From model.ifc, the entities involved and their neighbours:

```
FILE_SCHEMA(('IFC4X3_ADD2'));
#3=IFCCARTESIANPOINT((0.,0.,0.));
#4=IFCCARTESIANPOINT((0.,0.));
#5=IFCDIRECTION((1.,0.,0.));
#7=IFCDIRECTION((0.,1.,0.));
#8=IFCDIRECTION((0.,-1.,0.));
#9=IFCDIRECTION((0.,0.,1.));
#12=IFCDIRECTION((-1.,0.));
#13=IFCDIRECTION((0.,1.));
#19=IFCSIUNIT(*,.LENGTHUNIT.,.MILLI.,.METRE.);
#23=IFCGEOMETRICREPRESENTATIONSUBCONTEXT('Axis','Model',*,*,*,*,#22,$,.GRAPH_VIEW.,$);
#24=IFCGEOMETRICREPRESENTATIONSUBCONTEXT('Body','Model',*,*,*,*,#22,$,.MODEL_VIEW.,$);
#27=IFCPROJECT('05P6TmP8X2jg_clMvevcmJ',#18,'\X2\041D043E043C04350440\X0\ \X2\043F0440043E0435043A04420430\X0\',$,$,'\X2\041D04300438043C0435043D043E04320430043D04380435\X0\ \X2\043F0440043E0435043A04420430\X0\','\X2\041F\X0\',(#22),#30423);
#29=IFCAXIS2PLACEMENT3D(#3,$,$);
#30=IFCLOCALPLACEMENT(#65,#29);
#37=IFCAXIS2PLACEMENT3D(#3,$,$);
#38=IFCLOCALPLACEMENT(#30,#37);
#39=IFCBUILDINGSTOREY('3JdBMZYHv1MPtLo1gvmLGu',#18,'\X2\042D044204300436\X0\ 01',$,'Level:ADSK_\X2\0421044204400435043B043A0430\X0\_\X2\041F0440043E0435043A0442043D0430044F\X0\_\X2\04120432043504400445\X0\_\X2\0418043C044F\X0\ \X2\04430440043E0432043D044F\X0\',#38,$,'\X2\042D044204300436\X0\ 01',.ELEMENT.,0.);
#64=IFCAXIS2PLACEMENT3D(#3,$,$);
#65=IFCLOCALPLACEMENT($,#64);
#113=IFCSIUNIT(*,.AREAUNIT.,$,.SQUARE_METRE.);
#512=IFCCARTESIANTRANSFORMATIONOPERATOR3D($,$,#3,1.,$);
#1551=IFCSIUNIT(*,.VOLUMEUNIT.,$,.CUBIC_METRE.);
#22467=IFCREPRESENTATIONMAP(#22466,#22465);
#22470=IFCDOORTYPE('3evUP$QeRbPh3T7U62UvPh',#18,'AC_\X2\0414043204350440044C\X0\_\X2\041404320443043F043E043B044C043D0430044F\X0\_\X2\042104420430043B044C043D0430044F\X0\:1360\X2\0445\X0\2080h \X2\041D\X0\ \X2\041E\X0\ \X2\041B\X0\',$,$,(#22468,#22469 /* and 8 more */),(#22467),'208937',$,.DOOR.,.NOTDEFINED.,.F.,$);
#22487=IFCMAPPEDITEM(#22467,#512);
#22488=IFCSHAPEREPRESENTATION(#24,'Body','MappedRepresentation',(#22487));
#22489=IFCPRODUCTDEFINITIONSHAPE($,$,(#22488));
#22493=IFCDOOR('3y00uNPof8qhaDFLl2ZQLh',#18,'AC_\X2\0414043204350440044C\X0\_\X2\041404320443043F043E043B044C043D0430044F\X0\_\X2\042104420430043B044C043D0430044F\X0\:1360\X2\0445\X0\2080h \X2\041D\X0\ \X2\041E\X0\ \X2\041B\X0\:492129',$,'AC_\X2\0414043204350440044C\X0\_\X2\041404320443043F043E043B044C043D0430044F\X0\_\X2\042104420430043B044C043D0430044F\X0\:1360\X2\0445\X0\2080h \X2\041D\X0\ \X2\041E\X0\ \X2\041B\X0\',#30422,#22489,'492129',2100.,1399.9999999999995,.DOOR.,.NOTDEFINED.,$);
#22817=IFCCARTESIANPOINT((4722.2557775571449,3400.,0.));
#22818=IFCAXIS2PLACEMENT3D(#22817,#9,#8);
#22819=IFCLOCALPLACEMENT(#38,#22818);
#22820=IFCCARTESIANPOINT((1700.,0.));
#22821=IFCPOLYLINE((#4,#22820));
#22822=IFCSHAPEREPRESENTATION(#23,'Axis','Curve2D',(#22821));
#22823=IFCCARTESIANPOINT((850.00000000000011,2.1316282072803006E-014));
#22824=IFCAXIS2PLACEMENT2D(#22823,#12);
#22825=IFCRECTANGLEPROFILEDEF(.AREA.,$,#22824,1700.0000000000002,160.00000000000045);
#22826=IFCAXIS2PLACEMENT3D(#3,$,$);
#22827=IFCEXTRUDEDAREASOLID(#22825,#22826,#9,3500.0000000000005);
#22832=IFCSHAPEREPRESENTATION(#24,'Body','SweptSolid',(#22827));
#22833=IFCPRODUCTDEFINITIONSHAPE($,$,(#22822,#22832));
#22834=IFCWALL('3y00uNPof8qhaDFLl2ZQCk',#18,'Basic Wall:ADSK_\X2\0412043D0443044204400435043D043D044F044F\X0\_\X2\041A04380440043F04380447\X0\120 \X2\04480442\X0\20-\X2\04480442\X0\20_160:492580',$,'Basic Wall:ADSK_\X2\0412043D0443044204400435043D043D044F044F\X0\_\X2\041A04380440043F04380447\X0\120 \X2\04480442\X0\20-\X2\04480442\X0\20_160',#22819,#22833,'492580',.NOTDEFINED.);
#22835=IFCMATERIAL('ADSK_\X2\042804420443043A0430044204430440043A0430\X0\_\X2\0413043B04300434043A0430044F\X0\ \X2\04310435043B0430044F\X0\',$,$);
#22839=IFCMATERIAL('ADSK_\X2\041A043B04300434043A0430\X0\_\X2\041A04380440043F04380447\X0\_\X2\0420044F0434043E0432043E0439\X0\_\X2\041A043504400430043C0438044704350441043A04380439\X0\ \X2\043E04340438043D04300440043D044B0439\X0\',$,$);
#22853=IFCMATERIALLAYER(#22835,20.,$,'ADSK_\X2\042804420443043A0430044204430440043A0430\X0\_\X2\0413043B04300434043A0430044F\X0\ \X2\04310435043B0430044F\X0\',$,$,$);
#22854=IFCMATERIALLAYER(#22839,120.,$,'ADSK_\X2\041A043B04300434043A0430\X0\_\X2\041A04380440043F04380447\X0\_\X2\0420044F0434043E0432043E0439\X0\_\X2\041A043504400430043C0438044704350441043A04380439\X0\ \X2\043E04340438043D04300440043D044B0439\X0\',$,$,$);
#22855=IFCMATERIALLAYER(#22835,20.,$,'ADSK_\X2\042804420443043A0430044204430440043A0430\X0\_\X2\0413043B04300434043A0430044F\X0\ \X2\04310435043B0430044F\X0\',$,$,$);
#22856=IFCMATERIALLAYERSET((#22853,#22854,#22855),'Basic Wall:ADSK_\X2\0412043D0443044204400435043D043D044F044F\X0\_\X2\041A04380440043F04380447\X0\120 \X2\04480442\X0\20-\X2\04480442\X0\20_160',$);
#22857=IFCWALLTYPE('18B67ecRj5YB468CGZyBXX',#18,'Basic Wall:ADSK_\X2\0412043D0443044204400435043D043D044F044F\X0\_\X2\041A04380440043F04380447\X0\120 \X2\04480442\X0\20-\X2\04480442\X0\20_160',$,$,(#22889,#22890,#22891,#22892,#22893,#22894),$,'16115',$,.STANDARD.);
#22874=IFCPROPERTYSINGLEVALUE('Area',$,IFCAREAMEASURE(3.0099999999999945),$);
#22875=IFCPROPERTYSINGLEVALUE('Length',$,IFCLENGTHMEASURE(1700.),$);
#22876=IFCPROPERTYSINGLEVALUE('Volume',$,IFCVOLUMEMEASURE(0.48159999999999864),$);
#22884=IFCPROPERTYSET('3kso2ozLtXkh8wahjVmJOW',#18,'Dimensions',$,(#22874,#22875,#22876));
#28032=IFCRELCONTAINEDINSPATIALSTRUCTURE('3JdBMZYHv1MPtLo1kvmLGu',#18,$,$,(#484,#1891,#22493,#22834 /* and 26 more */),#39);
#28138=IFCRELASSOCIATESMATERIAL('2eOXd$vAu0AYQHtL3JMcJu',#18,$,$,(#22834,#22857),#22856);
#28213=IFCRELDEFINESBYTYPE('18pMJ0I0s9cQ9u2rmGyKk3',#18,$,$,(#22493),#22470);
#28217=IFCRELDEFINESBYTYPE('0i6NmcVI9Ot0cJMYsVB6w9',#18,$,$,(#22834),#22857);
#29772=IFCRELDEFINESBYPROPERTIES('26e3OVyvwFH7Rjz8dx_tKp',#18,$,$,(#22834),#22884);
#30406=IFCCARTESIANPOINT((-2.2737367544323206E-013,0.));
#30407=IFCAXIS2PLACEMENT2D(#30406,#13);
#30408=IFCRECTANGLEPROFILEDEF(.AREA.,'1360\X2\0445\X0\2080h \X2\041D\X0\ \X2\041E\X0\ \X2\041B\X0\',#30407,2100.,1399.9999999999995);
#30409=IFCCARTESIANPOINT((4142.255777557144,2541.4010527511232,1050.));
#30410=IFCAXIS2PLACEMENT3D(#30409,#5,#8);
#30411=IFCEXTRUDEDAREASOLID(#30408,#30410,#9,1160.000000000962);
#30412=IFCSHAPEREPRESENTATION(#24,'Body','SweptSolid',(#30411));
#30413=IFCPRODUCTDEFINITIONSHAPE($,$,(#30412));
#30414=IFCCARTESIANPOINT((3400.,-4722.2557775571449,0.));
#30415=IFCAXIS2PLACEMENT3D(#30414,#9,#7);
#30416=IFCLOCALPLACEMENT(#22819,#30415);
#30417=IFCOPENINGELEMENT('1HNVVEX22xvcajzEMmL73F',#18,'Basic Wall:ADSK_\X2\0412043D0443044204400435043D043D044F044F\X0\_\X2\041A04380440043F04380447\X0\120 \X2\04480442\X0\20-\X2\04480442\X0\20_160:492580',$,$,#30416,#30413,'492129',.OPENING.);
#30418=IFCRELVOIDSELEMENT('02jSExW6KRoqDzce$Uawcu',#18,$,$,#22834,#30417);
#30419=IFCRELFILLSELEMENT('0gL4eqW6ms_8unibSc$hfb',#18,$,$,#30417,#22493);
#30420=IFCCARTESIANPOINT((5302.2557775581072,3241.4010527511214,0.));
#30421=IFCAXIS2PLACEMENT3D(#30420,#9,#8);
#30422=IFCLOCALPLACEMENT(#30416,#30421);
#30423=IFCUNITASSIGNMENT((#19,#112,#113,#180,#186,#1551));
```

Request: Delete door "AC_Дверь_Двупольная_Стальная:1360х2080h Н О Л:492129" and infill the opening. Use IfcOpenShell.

```python
import ifcopenshell
import ifcopenshell.api.feature
import ifcopenshell.api.pset
import ifcopenshell.api.root
import ifcopenshell.geom
import ifcopenshell.util.element
import ifcopenshell.util.shape
import ifcopenshell.util.unit

model = ifcopenshell.open("model.ifc")
area_scale = ifcopenshell.util.unit.calculate_unit_scale(model, "AREAUNIT")
volume_scale = ifcopenshell.util.unit.calculate_unit_scale(model, "VOLUMEUNIT")
settings = ifcopenshell.geom.settings()


def volume(element):
    """Net volume in cubic metres, openings subtracted."""
    shape = ifcopenshell.geom.create_shape(settings, element)
    return ifcopenshell.util.shape.get_volume(shape.geometry)


door = model.by_id(22493)
opening = door.FillsVoids[0].RelatingOpeningElement
wall = opening.VoidsElements[0].RelatingBuildingElement
before = volume(wall)

ifcopenshell.api.root.remove_product(model, product=door)
ifcopenshell.api.feature.remove_feature(model, feature=opening)

after = volume(wall)
thickness = 0.16  # wall thickness in metres

# Update the wall's stored quantities.
pset = model.by_id(ifcopenshell.util.element.get_pset(wall, "Dimensions", should_inherit=False)["id"])
ifcopenshell.api.pset.edit_pset(model, pset=pset, properties={
    "Area": model.create_entity("IfcAreaMeasure", after / thickness / area_scale),
    "Volume": model.create_entity("IfcVolumeMeasure", after / volume_scale),
})

print(f"wall volume {before:.3f} -> {after:.3f} m3")

model.write("model_edited.ifc")
```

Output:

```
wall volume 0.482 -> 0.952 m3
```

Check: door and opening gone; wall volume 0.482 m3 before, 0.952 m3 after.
